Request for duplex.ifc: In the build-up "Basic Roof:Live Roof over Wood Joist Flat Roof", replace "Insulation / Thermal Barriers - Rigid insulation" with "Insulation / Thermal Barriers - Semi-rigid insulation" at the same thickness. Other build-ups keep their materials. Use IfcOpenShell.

First a look at what the model holds.

```python
import ifcopenshell
import ifcopenshell.util.element

model = ifcopenshell.open("duplex.ifc")
print(model.schema)
for layer_set in model.by_type("IfcMaterialLayerSet"):
    if layer_set.LayerSetName == "Basic Roof:Live Roof over Wood Joist Flat Roof":
        for layer in layer_set.MaterialLayers:
            print(layer.id(), layer.Material and layer.Material.Name, layer.LayerThickness, sep=" | ")
        print(len(ifcopenshell.util.element.get_elements_by_material(model, layer_set)), "elements and types use it")
print(sorted(m.Name for m in model.by_type("IfcMaterial") if m.Name)[:60])
```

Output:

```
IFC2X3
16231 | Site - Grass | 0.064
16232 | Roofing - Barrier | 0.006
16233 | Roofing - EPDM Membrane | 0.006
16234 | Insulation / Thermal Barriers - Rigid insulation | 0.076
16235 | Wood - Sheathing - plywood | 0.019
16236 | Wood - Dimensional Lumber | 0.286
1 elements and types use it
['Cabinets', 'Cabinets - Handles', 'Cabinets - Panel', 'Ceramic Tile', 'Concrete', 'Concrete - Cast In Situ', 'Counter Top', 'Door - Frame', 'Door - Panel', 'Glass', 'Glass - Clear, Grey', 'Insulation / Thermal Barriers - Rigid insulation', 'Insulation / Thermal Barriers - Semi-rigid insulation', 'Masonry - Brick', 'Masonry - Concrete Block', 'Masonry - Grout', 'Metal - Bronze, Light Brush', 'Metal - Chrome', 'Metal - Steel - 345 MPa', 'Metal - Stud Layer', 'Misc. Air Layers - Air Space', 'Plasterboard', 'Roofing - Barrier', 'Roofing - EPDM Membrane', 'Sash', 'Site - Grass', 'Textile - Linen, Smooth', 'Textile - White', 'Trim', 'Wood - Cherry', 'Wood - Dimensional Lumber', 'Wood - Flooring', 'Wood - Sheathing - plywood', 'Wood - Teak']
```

```python
import ifcopenshell
import ifcopenshell.api.material

model = ifcopenshell.open("duplex.ifc")

layer_set = next(s for s in model.by_type("IfcMaterialLayerSet") if s.LayerSetName == "Basic Roof:Live Roof over Wood Joist Flat Roof")
layer = next(l for l in layer_set.MaterialLayers if l.Material and l.Material.Name == "Insulation / Thermal Barriers - Rigid insulation")
material = next(m for m in model.by_type("IfcMaterial") if m.Name == "Insulation / Thermal Barriers - Semi-rigid insulation")

# Point this one layer at the other material; renaming the old one would change it everywhere.
ifcopenshell.api.material.edit_layer(model, layer=layer, attributes={}, material=material)

print([l.Material.Name if l.Material else None for l in layer_set.MaterialLayers])

model.write("duplex-out.ifc")
```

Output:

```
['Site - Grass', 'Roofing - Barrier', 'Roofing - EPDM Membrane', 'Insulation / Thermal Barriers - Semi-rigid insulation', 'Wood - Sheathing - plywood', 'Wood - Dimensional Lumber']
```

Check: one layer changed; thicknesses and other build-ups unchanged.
